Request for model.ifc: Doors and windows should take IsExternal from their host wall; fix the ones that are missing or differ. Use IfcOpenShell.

First a look at what the model holds.

```python
import ifcopenshell
import ifcopenshell.util.element

model = ifcopenshell.open("model.ifc")
print(model.schema)
seen = {}
for e in model.by_type("IfcDoor") + model.by_type("IfcWindow"):
    if not e.FillsVoids:
        continue
    host = e.FillsVoids[0].RelatingOpeningElement.VoidsElements[0].RelatingBuildingElement
    own = ifcopenshell.util.element.get_pset(e, f"Pset_{e.is_a()[3:].removesuffix('StandardCase')}Common", "IsExternal")
    wall = ifcopenshell.util.element.get_pset(host, "Pset_WallCommon", "IsExternal")
    seen[e.is_a(), own, wall] = seen.get((e.is_a(), own, wall), 0) + 1
for (cls, own, wall), count in sorted(seen.items(), key=str):
    print(count, cls, "IsExternal:", own, "| host wall:", wall)
```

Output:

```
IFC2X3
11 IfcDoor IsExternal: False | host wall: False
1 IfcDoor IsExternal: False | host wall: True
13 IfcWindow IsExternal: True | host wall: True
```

```python
import ifcopenshell
import ifcopenshell.api.pset
import ifcopenshell.util.element

model = ifcopenshell.open("model.ifc")

count = 0
for ifc_class, pset_name in (("IfcDoor", "Pset_DoorCommon"), ("IfcWindow", "Pset_WindowCommon")):
    for e in model.by_type(ifc_class):
        if not e.FillsVoids:
            continue
        host = e.FillsVoids[0].RelatingOpeningElement.VoidsElements[0].RelatingBuildingElement
        external = ifcopenshell.util.element.get_pset(host, "Pset_WallCommon", "IsExternal")
        if external is None or ifcopenshell.util.element.get_pset(e, pset_name, "IsExternal") == external:
            continue
        pset = ifcopenshell.api.pset.add_pset(model, product=e, name=pset_name)
        ifcopenshell.api.pset.edit_pset(model, pset=pset, properties={"IsExternal": external})
        count += 1

print(count, "updated")

model.write("model-out.ifc")
```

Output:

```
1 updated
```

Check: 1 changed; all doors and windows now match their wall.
